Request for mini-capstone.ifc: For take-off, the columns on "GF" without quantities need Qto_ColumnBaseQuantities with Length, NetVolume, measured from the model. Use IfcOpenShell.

First a look at what the model holds.

```python
import ifcopenshell
import ifcopenshell.util.element
import ifcopenshell.util.unit

model = ifcopenshell.open("mini-capstone.ifc")
print(model.schema)
for unit_type in ("LENGTHUNIT", "AREAUNIT", "VOLUMEUNIT"):
    print(unit_type, ifcopenshell.util.unit.calculate_unit_scale(model, unit_type))
storey = next(s for s in model.by_type("IfcBuildingStorey") if s.Name == "GF")
columns = [e for e in ifcopenshell.util.element.get_decomposition(storey) if e.is_a("IfcColumn")]
for e in sorted(columns, key=lambda e: e.id()):
    print(e.id(), e.is_a(), e.Name, list(ifcopenshell.util.element.get_psets(e, qtos_only=True)), sep=" | ")
```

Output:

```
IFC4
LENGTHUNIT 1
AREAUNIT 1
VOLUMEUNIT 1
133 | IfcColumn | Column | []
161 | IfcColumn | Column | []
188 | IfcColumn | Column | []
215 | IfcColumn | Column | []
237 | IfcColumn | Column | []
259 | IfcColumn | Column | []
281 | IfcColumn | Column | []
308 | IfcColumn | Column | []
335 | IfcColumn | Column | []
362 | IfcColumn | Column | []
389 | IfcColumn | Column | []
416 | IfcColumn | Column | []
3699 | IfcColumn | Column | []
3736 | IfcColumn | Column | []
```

```python
import ifcopenshell
import ifcopenshell.api.pset
import ifcopenshell.geom
import ifcopenshell.util.element
import ifcopenshell.util.shape
import ifcopenshell.util.unit

model = ifcopenshell.open("mini-capstone.ifc")
unit_scale = ifcopenshell.util.unit.calculate_unit_scale(model)
volume_scale = ifcopenshell.util.unit.calculate_unit_scale(model, "VOLUMEUNIT")
settings = ifcopenshell.geom.settings()

storey = next(s for s in model.by_type("IfcBuildingStorey") if s.Name == "GF")
columns = [e for e in ifcopenshell.util.element.get_decomposition(storey) if e.is_a("IfcColumn")]

for e in sorted(columns, key=lambda e: e.id()):
    if ifcopenshell.util.element.get_psets(e, qtos_only=True, should_inherit=False):
        continue
    # Geometry comes back in metres, in the element's own axes.
    shape = ifcopenshell.geom.create_shape(settings, e)
    values = {
        "Length": ifcopenshell.util.shape.get_z(shape.geometry) / unit_scale,
        "NetVolume": ifcopenshell.util.shape.get_volume(shape.geometry) / volume_scale,
    }
    qto = ifcopenshell.api.pset.add_qto(model, product=e, name="Qto_ColumnBaseQuantities")
    ifcopenshell.api.pset.edit_qto(model, qto=qto, properties=values)
    print(e.id(), {k: round(v, 3) for k, v in values.items()})

model.write("mini-capstone_rev.ifc")
```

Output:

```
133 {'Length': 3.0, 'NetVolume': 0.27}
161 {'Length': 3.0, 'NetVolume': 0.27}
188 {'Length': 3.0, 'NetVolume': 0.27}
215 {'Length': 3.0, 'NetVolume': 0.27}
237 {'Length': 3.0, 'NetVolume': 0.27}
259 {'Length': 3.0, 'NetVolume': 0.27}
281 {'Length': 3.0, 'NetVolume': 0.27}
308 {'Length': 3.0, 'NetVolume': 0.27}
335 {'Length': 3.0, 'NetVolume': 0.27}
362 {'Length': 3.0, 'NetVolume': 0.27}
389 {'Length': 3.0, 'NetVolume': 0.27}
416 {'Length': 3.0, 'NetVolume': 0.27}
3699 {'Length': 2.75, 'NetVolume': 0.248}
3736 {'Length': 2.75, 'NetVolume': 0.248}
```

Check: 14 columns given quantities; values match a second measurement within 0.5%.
